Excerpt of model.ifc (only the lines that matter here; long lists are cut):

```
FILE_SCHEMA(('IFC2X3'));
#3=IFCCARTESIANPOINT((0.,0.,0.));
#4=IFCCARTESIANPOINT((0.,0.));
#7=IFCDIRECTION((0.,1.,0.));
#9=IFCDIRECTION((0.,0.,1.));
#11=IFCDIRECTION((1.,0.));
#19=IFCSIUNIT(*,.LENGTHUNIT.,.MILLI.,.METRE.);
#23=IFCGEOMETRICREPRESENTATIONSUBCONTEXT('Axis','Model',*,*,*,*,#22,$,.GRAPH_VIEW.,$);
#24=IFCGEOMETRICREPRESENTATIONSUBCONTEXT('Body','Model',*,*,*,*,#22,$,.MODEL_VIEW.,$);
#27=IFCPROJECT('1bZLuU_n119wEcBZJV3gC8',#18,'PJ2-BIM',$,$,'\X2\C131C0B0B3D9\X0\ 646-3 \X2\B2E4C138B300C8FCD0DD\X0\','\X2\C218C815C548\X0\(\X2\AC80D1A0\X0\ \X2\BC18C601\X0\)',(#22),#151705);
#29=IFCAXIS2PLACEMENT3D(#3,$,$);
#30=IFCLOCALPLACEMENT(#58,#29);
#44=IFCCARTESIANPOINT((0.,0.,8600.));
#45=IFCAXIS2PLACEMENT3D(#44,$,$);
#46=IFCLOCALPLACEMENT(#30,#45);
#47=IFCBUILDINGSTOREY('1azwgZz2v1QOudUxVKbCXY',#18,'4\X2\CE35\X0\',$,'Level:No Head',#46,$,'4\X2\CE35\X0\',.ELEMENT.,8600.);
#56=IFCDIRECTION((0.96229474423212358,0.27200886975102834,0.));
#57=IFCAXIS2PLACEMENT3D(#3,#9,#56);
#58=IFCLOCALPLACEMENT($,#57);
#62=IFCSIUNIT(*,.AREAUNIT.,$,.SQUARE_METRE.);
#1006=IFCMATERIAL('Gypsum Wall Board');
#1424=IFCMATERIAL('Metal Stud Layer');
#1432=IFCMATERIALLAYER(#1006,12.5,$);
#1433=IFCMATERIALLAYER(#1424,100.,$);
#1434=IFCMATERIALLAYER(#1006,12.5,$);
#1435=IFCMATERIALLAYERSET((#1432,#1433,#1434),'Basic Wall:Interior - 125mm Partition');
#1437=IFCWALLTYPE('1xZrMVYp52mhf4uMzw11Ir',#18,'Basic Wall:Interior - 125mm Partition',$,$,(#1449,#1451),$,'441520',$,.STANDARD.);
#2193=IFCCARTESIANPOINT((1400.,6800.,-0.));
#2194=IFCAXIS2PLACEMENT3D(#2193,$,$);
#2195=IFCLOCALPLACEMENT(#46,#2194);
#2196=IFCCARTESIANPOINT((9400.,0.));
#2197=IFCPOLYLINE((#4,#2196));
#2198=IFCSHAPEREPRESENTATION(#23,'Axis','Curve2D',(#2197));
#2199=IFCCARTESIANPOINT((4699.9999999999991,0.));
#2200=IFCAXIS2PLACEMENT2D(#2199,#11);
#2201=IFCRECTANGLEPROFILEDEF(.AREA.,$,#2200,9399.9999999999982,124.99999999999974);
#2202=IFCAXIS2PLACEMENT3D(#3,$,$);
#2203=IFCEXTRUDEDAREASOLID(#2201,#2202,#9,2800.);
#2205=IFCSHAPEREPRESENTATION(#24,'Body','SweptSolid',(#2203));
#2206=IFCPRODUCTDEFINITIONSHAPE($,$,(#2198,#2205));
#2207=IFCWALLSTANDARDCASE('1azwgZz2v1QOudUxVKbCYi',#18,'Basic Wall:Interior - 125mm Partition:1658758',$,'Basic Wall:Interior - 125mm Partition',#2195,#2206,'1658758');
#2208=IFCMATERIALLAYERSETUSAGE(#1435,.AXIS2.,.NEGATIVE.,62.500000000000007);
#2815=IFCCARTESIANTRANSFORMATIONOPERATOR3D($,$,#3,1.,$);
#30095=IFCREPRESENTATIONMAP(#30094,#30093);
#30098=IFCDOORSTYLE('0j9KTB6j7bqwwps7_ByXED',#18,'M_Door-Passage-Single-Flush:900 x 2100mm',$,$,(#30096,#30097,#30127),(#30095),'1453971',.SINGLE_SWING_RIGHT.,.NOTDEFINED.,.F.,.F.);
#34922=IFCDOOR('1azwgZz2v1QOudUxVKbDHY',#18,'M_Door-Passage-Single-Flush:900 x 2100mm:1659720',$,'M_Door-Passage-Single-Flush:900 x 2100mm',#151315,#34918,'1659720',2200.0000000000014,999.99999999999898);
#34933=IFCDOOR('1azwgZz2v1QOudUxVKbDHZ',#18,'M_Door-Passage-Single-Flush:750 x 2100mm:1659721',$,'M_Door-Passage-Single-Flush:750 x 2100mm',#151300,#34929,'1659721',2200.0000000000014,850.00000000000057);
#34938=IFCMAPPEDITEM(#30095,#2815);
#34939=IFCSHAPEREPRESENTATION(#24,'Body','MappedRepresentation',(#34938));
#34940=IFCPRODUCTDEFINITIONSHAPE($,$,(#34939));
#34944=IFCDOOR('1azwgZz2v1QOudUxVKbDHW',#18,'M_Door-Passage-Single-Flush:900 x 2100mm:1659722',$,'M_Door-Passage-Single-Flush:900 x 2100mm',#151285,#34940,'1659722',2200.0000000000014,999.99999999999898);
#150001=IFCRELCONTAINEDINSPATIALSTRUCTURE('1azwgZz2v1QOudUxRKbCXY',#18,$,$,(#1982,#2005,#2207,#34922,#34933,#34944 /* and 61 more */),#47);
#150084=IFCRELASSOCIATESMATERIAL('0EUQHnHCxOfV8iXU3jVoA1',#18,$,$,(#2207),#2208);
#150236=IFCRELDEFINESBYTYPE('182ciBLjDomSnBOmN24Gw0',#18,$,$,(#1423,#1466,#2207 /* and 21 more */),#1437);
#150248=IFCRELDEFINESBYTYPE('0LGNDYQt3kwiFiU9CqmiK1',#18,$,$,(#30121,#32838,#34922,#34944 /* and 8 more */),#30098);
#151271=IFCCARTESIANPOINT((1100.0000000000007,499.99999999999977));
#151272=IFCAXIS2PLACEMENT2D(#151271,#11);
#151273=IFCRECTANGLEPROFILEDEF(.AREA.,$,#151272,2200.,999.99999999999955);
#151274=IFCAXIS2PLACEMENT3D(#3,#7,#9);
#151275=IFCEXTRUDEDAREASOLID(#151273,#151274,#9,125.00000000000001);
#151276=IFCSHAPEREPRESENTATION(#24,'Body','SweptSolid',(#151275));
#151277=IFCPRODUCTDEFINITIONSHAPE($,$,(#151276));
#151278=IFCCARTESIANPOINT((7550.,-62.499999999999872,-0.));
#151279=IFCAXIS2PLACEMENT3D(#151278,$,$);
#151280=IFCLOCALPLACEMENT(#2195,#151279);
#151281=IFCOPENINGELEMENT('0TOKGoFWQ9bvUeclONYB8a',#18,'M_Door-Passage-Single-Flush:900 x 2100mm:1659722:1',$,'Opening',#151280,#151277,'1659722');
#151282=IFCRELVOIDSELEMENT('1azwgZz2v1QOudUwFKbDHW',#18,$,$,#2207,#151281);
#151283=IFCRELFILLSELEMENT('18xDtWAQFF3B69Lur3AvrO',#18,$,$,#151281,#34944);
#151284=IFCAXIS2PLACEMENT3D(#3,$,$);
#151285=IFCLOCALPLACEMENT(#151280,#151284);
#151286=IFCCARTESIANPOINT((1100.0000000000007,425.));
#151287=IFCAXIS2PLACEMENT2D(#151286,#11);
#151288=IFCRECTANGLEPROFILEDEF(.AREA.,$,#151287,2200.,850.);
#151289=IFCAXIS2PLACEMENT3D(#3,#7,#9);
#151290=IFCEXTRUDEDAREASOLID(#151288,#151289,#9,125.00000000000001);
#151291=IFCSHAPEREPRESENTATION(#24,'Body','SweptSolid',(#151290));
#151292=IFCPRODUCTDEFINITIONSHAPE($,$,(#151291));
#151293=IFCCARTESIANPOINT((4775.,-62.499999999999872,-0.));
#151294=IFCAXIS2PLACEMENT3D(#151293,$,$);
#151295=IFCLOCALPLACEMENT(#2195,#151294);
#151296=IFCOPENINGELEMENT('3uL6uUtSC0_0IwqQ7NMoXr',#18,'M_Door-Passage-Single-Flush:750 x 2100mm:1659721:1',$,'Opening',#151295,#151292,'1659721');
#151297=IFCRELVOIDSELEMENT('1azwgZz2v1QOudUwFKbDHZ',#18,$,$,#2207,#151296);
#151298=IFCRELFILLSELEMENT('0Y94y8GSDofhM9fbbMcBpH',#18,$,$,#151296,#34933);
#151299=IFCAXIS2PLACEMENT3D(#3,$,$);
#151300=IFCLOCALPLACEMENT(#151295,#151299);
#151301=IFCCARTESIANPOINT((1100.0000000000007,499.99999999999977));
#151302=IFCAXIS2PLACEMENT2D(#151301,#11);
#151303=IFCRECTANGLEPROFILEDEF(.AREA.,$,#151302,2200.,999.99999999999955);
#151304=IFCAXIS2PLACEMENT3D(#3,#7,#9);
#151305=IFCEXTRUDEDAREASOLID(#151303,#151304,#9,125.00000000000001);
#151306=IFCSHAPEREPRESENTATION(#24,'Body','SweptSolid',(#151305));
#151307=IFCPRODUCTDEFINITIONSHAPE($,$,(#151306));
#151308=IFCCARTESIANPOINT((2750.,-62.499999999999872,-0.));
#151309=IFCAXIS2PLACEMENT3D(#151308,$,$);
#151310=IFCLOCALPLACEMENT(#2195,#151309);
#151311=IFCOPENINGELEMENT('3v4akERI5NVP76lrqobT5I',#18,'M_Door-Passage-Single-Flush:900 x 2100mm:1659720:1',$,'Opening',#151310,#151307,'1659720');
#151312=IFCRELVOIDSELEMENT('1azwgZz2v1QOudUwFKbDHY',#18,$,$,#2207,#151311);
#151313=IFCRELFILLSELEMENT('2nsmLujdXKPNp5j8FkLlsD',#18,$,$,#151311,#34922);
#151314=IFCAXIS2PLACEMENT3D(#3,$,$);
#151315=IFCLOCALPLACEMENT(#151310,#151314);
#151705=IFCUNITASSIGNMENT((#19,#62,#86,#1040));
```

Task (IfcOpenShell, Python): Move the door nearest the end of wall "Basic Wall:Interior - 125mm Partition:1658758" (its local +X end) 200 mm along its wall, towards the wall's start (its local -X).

```python
import ifcopenshell
import ifcopenshell.api.geometry
import ifcopenshell.util.placement

model = ifcopenshell.open("model.ifc")

door = model.by_guid("1azwgZz2v1QOudUxVKbDHW")
opening = door.FillsVoids[0].RelatingOpeningElement
wall = opening.VoidsElements[0].RelatingBuildingElement

wall_matrix = ifcopenshell.util.placement.get_local_placement(wall.ObjectPlacement)
shift = wall_matrix[:3, 0] * -200.0
before = ifcopenshell.util.placement.get_local_placement(door.ObjectPlacement)[:3, 3].copy()

# The door is placed relative to its opening, so it follows when the opening moves.
matrix = ifcopenshell.util.placement.get_local_placement(opening.ObjectPlacement)
matrix[:3, 3] += shift
ifcopenshell.api.geometry.edit_object_placement(
    model, product=opening, matrix=matrix, is_si=False, should_transform_children=True
)

after = ifcopenshell.util.placement.get_local_placement(door.ObjectPlacement)[:3, 3]
print("door moved by", (after - before).round(3) + 0.0)

model.write("model_edited.ifc")
```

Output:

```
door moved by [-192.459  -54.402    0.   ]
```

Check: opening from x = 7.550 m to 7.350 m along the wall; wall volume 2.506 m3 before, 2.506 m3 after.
